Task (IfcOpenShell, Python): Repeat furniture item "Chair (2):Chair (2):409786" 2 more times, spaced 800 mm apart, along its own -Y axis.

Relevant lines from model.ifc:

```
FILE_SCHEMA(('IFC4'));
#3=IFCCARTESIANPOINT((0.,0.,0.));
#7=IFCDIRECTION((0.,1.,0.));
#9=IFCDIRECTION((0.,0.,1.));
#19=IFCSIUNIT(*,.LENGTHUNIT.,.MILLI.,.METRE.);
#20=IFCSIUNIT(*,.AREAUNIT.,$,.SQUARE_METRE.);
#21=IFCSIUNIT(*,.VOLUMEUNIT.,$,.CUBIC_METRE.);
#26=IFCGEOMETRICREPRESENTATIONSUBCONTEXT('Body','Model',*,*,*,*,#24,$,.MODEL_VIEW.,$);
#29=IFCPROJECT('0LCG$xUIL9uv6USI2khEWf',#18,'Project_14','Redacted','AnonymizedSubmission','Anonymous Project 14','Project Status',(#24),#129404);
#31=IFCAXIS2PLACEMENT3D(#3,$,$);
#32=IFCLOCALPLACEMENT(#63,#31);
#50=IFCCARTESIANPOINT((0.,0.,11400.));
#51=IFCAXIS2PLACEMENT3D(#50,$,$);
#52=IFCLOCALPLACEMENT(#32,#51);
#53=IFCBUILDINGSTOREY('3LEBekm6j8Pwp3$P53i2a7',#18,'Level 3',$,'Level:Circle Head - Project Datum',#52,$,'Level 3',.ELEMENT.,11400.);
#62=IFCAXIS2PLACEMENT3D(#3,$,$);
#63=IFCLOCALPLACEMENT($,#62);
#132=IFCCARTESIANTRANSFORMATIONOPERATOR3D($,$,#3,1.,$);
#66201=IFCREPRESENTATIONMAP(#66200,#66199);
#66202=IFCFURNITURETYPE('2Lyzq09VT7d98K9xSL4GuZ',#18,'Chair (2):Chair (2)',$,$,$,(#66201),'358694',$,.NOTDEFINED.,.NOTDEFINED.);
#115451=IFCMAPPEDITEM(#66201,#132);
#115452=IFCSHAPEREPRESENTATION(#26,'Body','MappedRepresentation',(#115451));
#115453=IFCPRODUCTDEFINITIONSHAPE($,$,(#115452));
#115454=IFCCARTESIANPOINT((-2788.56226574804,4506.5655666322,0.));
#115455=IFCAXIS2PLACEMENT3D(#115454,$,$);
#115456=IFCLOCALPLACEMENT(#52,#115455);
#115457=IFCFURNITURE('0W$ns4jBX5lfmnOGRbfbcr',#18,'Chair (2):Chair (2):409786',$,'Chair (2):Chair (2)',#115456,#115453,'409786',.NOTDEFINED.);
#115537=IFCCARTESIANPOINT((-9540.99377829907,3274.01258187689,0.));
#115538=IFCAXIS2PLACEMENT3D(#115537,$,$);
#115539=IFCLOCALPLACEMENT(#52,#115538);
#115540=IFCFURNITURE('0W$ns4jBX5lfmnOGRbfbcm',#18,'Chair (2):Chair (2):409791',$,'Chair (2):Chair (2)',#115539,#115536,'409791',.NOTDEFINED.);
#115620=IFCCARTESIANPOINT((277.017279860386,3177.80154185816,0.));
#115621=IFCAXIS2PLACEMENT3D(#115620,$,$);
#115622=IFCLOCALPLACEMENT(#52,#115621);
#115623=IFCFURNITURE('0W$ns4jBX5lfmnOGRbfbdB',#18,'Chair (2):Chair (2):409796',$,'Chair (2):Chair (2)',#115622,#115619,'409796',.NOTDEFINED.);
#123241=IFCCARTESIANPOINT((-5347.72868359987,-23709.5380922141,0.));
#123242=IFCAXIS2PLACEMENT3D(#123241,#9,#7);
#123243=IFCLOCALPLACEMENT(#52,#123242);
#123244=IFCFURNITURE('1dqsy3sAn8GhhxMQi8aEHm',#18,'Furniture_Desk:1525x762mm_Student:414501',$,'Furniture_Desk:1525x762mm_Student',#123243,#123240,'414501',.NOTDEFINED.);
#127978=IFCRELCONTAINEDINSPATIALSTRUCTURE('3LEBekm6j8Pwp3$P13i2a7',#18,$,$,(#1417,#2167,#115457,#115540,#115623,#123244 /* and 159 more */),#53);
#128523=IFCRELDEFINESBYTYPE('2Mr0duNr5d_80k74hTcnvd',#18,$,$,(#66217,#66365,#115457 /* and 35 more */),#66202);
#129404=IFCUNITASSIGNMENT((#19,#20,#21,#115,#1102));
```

```python
import ifcopenshell
import ifcopenshell.api.geometry
import ifcopenshell.api.root
import ifcopenshell.util.element
import ifcopenshell.util.placement
import ifcopenshell.util.unit

model = ifcopenshell.open("model.ifc")
unit_scale = ifcopenshell.util.unit.calculate_unit_scale(model)


def reuse_history(source, copy):
    """copy_class also copies each property set's owner history, people and application; keep the originals."""
    for rel in copy.IsDefinedBy:
        if rel.is_a("IfcRelDefinesByProperties") and (history := rel.RelatingPropertyDefinition.OwnerHistory):
            rel.RelatingPropertyDefinition.OwnerHistory = source.OwnerHistory
            ifcopenshell.util.element.remove_deep2(model, history)


source = model.by_id(115457)
base = ifcopenshell.util.placement.get_local_placement(source.ObjectPlacement)
step = -base[:3, 1] * 0.8 / unit_scale

for i in range(1, 3):
    copy = ifcopenshell.api.root.copy_class(model, product=source)
    copy.Representation = ifcopenshell.util.element.copy_deep(
        model, source.Representation, exclude=["IfcGeometricRepresentationContext", "IfcRepresentationMap"]
    )
    copy.Name = "Chair (2):Chair (2)"
    copy.Tag = None
    reuse_history(source, copy)
    matrix = base.copy()
    matrix[:3, 3] += i * step
    print("added at", matrix[:3, 3].round(3) + 0.0)
    ifcopenshell.api.geometry.edit_object_placement(model, product=copy, matrix=matrix, is_si=False)

model.write("model_updated.ifc")
```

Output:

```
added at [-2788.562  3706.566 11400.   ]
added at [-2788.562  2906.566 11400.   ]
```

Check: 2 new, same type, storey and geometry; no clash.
